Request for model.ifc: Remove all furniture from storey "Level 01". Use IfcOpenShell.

First a look at what the model holds.

```python
import ifcopenshell
import ifcopenshell.util.element

model = ifcopenshell.open("model.ifc")
print(model.schema)
storey = next(s for s in model.by_type("IfcBuildingStorey") if s.Name == "Level 01")
furniture = [e for e in ifcopenshell.util.element.get_decomposition(storey) if e.is_a("IfcFurnishingElement")]
seen = {}
for e in furniture:
    element_type = ifcopenshell.util.element.get_type(e)
    name = element_type.Name if element_type not in (None, e) else None
    seen[name] = seen.get(name, 0) + 1
for name, count in sorted(seen.items(), key=str):
    print(count, "x", name)
```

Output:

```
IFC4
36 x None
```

```python
import ifcopenshell
import ifcopenshell.api.root
import ifcopenshell.util.element

model = ifcopenshell.open("model.ifc")

storey = next(s for s in model.by_type("IfcBuildingStorey") if s.Name == "Level 01")
furniture = [e for e in ifcopenshell.util.element.get_decomposition(storey) if e.is_a("IfcFurnishingElement")]

for e in furniture:
    ifcopenshell.api.root.remove_product(model, product=e)
print(len(furniture), "removed")

model.write("model_updated.ifc")
```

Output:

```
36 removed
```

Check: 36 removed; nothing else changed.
